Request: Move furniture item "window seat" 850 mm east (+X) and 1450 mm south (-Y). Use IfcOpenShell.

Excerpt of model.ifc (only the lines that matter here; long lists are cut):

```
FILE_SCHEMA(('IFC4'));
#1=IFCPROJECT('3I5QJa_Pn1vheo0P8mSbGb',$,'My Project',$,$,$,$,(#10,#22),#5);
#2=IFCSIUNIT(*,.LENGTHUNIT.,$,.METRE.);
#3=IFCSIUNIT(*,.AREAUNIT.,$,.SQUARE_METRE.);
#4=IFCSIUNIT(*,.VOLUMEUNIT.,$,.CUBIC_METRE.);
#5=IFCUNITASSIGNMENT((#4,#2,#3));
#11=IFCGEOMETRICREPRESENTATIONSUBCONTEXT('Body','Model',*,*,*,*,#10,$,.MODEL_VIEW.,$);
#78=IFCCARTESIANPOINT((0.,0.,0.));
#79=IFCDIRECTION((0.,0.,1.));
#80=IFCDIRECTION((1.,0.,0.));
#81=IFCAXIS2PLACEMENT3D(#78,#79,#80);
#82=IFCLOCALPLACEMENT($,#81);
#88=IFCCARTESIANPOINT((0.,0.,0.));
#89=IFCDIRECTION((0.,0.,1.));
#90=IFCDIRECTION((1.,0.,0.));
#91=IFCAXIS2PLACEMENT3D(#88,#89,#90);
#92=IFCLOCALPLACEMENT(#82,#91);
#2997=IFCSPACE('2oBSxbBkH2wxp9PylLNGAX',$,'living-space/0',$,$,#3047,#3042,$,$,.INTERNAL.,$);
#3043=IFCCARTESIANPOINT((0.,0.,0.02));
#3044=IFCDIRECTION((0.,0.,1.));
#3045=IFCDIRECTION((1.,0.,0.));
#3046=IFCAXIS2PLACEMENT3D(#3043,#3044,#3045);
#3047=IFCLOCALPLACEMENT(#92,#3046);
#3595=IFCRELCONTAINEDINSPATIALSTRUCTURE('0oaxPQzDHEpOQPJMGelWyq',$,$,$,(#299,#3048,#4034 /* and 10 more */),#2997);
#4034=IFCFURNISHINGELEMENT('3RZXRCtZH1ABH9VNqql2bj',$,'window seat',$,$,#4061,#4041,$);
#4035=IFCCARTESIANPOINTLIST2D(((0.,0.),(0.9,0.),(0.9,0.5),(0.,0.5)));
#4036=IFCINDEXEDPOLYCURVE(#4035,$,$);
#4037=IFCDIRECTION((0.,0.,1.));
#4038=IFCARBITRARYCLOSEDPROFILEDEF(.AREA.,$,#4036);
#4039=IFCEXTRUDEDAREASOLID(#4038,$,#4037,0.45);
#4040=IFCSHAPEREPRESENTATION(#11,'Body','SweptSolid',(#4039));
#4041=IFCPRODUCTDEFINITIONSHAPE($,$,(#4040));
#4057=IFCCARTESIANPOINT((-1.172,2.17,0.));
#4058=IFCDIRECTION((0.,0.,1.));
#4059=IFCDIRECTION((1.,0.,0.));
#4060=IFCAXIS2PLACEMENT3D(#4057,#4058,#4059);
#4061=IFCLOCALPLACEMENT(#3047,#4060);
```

```python
import ifcopenshell
import ifcopenshell.api.geometry
import ifcopenshell.util.placement
import ifcopenshell.util.unit

model = ifcopenshell.open("model.ifc")
unit_scale = ifcopenshell.util.unit.calculate_unit_scale(model)

item = model.by_guid("3RZXRCtZH1ABH9VNqql2bj")
matrix = ifcopenshell.util.placement.get_local_placement(item.ObjectPlacement)
matrix[0, 3] += 0.85 / unit_scale
matrix[1, 3] -= 1.45 / unit_scale
ifcopenshell.api.geometry.edit_object_placement(model, product=item, matrix=matrix, is_si=False)

print(ifcopenshell.util.placement.get_local_placement(item.ObjectPlacement).round(3) + 0.0)

model.write("model_rev.ifc")
```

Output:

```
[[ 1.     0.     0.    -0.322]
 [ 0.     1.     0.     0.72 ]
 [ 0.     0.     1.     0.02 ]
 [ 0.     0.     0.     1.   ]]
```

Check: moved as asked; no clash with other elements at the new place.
